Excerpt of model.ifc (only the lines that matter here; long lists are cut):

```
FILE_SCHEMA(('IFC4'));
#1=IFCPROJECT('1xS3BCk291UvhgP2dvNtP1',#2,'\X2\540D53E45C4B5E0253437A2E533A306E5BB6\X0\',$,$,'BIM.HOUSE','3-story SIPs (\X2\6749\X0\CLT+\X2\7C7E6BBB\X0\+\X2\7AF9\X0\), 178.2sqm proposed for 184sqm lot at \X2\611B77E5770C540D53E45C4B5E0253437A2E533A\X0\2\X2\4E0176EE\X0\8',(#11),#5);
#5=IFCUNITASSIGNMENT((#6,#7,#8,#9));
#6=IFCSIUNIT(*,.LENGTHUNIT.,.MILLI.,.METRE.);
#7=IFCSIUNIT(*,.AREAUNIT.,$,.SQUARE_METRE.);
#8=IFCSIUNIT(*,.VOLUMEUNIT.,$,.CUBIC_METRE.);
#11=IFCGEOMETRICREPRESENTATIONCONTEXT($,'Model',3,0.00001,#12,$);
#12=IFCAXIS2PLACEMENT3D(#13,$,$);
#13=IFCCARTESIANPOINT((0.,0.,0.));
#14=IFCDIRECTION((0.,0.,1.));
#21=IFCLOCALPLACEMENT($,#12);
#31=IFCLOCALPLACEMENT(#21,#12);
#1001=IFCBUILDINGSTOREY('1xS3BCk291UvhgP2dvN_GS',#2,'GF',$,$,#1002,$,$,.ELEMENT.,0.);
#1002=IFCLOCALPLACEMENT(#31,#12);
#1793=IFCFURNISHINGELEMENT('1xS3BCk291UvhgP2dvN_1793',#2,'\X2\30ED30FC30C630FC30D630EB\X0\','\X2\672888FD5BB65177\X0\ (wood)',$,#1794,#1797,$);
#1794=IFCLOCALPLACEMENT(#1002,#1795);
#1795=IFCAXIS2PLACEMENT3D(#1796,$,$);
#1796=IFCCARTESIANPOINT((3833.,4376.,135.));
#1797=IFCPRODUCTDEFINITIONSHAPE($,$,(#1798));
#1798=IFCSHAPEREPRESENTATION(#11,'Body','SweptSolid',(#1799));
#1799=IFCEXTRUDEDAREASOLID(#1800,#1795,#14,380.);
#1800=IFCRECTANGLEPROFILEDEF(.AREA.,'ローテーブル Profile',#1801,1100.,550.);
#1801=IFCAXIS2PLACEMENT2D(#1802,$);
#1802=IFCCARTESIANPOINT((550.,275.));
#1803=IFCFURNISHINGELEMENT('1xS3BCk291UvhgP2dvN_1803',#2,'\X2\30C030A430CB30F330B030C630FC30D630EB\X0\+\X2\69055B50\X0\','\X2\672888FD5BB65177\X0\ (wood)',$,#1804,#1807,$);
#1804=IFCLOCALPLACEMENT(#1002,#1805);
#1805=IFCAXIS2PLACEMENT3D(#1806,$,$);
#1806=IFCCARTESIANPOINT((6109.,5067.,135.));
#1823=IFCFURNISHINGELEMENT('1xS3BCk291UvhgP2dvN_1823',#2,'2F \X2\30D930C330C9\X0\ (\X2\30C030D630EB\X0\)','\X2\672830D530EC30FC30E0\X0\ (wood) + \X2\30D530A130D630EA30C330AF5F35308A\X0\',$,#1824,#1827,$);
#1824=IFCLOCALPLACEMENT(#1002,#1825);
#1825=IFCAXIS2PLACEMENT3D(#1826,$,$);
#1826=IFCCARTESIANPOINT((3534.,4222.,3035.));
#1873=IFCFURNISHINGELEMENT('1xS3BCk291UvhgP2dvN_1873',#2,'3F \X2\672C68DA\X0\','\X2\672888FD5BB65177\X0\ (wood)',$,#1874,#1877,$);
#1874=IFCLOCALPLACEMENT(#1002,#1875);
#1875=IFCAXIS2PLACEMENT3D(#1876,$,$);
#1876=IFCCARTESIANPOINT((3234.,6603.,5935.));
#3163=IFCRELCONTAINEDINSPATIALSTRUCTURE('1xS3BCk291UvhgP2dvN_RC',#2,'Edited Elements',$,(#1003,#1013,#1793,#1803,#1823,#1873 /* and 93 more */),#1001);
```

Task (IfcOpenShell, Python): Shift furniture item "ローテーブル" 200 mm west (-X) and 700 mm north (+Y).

```python
import ifcopenshell
import ifcopenshell.api.geometry
import ifcopenshell.util.placement

model = ifcopenshell.open("model.ifc")

item = model.by_id(1793)
matrix = ifcopenshell.util.placement.get_local_placement(item.ObjectPlacement)
matrix[0, 3] -= 200.0
matrix[1, 3] += 700.0
ifcopenshell.api.geometry.edit_object_placement(model, product=item, matrix=matrix, is_si=False)

print(ifcopenshell.util.placement.get_local_placement(item.ObjectPlacement).round(3) + 0.0)

model.write("model_rev.ifc")
```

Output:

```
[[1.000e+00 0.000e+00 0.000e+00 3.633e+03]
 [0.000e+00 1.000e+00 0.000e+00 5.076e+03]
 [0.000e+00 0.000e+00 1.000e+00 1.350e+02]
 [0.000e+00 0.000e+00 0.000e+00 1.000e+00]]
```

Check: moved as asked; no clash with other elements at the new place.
